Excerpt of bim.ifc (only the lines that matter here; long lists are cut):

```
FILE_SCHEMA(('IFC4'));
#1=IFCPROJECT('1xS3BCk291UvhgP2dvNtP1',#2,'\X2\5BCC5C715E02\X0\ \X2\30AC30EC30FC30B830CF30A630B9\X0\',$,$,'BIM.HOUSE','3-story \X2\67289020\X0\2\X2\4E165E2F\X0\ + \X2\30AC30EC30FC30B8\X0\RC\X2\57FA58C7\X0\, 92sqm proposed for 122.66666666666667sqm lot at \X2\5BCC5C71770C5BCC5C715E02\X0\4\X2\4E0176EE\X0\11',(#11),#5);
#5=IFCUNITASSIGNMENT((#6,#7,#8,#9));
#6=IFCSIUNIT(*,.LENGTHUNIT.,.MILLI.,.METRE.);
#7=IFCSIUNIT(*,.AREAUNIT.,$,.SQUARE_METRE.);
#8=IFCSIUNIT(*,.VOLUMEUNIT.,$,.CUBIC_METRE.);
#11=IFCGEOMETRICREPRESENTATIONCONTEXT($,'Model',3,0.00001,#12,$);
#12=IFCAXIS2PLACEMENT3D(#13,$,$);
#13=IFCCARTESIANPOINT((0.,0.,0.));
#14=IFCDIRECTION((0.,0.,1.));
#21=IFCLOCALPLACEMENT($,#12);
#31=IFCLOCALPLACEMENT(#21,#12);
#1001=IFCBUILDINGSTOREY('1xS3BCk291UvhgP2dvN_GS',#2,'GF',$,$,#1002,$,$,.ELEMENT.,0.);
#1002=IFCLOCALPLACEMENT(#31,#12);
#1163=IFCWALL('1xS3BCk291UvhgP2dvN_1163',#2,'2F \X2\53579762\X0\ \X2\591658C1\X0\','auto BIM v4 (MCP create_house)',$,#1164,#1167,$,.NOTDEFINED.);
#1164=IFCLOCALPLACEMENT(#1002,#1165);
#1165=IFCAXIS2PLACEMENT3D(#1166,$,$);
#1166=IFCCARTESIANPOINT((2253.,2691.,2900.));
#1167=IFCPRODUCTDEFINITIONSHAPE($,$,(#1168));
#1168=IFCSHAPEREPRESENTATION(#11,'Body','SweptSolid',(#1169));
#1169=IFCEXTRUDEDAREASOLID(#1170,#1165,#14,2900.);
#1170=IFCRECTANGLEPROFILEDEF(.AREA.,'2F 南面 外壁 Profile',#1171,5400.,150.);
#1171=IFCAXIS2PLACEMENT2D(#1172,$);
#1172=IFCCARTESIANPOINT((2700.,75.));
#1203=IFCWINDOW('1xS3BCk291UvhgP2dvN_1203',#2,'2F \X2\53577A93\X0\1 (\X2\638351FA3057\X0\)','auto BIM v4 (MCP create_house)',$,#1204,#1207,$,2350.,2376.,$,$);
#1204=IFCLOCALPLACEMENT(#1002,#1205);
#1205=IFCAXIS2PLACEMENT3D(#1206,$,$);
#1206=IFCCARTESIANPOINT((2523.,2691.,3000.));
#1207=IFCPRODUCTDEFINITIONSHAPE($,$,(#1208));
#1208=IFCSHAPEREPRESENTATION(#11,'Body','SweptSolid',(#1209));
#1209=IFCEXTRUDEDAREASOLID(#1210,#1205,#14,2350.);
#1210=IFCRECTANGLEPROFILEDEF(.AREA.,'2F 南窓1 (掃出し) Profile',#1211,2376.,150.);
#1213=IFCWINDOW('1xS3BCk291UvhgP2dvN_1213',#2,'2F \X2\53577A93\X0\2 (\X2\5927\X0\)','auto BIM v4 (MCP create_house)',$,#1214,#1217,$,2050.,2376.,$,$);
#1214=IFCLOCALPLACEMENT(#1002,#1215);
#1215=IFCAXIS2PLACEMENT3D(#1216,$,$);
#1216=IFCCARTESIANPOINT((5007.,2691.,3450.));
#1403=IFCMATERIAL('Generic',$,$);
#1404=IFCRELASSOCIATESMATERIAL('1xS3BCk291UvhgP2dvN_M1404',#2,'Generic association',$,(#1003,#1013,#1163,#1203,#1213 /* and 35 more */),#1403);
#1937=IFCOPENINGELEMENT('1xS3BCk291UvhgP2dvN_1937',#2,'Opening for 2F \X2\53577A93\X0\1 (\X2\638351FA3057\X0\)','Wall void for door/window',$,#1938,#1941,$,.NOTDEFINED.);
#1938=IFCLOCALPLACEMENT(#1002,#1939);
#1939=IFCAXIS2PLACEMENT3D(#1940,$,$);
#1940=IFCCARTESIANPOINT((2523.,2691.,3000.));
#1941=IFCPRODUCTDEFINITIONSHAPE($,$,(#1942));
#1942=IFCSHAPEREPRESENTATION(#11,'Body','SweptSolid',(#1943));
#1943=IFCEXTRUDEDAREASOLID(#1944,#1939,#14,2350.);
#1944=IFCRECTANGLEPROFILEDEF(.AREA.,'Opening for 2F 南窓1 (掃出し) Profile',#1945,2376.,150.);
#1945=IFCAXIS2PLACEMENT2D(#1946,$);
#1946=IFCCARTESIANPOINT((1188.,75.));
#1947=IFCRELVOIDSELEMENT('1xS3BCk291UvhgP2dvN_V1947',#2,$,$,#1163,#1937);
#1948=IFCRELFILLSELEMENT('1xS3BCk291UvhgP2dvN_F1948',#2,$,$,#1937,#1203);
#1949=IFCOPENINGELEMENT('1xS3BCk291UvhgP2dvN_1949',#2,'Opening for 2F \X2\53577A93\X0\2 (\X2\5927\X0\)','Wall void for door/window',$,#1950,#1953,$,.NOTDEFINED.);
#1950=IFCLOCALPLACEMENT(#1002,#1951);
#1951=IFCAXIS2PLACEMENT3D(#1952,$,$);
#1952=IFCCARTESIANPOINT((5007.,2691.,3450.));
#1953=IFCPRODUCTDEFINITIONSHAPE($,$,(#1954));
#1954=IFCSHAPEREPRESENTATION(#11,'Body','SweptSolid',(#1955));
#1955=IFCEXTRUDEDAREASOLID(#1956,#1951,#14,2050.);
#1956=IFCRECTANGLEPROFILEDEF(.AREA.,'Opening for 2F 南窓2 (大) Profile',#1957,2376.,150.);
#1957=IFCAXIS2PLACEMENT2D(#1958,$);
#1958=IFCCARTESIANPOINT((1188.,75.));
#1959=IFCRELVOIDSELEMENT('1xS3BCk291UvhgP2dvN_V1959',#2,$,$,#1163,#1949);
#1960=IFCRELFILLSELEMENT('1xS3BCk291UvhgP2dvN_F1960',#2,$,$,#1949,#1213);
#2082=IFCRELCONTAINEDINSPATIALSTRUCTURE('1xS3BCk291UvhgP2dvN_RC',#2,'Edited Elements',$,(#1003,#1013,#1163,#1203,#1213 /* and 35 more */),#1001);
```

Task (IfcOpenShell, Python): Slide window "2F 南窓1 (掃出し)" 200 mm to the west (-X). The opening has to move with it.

```python
import ifcopenshell
import ifcopenshell.api.geometry
import ifcopenshell.util.placement
import ifcopenshell.util.unit

model = ifcopenshell.open("bim.ifc")
unit_scale = ifcopenshell.util.unit.calculate_unit_scale(model)

window = model.by_id(1203)
opening = window.FillsVoids[0].RelatingOpeningElement
wall = opening.VoidsElements[0].RelatingBuildingElement

wall_matrix = ifcopenshell.util.placement.get_local_placement(wall.ObjectPlacement)
shift = wall_matrix[:3, 0] * -0.2 / unit_scale
before = ifcopenshell.util.placement.get_local_placement(window.ObjectPlacement)[:3, 3].copy()

# The window is not placed relative to its opening, so move both.
for product in (opening, window):
    matrix = ifcopenshell.util.placement.get_local_placement(product.ObjectPlacement)
    matrix[:3, 3] += shift
    ifcopenshell.api.geometry.edit_object_placement(model, product=product, matrix=matrix, is_si=False)

after = ifcopenshell.util.placement.get_local_placement(window.ObjectPlacement)[:3, 3]
print("window moved by", (after - before).round(3) + 0.0)

model.write("bim_edited.ifc")
```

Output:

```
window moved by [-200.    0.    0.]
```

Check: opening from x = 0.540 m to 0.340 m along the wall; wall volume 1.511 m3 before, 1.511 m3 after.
